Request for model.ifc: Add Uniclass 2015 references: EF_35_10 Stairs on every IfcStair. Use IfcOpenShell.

First a look at what the model holds.

```python
import ifcopenshell

model = ifcopenshell.open("model.ifc")
print(model.schema)
print("classifications:", [c.Name for c in model.by_type("IfcClassification")])
for ifc_class in ("IfcDoor", "IfcRoof", "IfcStair", "IfcWall", "IfcWindow"):
    print(ifc_class, len(model.by_type(ifc_class)))
```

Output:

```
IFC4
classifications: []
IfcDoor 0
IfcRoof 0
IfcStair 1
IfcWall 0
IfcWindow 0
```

```python
import ifcopenshell
import ifcopenshell.api.classification

model = ifcopenshell.open("model.ifc")

system = ifcopenshell.api.classification.add_classification(model, classification="Uniclass 2015")

codes = {
    "IfcStair": ("EF_35_10", "Stairs"),
}
for ifc_class, (code, name) in codes.items():
    products = model.by_type(ifc_class)
    ifcopenshell.api.classification.add_reference(
        model, products=products, classification=system, identification=code, name=name
    )
    print(code, len(products))

model.write("model-out.ifc")
```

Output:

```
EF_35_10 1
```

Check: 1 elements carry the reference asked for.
